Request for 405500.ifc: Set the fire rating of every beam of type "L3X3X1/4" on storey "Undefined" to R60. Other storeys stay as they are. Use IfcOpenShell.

First a look at what the model holds.

```python
import ifcopenshell
import ifcopenshell.util.element

model = ifcopenshell.open("405500.ifc")
print(model.schema)
storey = next(s for s in model.by_type("IfcBuildingStorey") if s.Name == "Undefined")
beams = [e for e in ifcopenshell.util.element.get_decomposition(storey) if e.is_a("IfcBeam")]
seen = {}
for e in beams:
    element_type = ifcopenshell.util.element.get_type(e)
    key = (element_type.Name if element_type != e and element_type else None, ifcopenshell.util.element.get_pset(e, "Pset_BeamCommon", "FireRating"))
    seen[key] = seen.get(key, 0) + 1
for (name, value), count in sorted(seen.items(), key=str):
    print(count, "x", name, "|", value)
```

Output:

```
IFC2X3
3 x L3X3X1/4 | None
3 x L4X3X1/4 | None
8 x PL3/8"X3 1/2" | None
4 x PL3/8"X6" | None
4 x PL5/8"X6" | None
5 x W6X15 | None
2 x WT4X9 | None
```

```python
import ifcopenshell
import ifcopenshell.api.pset
import ifcopenshell.util.element

model = ifcopenshell.open("405500.ifc")

storey = next(s for s in model.by_type("IfcBuildingStorey") if s.Name == "Undefined")
beams = [e for e in ifcopenshell.util.element.get_decomposition(storey) if e.is_a("IfcBeam")]

count = 0
for e in beams:
    element_type = ifcopenshell.util.element.get_type(e)
    if element_type in (None, e) or element_type.Name != "L3X3X1/4":
        continue
    # add_pset returns the element's existing set when there is one.
    pset = ifcopenshell.api.pset.add_pset(model, product=e, name="Pset_BeamCommon")
    ifcopenshell.api.pset.edit_pset(model, pset=pset, properties={"FireRating": "R60"})
    count += 1

print(count, "beams updated")

model.write("405500-out.ifc")
```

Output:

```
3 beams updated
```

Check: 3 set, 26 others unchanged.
